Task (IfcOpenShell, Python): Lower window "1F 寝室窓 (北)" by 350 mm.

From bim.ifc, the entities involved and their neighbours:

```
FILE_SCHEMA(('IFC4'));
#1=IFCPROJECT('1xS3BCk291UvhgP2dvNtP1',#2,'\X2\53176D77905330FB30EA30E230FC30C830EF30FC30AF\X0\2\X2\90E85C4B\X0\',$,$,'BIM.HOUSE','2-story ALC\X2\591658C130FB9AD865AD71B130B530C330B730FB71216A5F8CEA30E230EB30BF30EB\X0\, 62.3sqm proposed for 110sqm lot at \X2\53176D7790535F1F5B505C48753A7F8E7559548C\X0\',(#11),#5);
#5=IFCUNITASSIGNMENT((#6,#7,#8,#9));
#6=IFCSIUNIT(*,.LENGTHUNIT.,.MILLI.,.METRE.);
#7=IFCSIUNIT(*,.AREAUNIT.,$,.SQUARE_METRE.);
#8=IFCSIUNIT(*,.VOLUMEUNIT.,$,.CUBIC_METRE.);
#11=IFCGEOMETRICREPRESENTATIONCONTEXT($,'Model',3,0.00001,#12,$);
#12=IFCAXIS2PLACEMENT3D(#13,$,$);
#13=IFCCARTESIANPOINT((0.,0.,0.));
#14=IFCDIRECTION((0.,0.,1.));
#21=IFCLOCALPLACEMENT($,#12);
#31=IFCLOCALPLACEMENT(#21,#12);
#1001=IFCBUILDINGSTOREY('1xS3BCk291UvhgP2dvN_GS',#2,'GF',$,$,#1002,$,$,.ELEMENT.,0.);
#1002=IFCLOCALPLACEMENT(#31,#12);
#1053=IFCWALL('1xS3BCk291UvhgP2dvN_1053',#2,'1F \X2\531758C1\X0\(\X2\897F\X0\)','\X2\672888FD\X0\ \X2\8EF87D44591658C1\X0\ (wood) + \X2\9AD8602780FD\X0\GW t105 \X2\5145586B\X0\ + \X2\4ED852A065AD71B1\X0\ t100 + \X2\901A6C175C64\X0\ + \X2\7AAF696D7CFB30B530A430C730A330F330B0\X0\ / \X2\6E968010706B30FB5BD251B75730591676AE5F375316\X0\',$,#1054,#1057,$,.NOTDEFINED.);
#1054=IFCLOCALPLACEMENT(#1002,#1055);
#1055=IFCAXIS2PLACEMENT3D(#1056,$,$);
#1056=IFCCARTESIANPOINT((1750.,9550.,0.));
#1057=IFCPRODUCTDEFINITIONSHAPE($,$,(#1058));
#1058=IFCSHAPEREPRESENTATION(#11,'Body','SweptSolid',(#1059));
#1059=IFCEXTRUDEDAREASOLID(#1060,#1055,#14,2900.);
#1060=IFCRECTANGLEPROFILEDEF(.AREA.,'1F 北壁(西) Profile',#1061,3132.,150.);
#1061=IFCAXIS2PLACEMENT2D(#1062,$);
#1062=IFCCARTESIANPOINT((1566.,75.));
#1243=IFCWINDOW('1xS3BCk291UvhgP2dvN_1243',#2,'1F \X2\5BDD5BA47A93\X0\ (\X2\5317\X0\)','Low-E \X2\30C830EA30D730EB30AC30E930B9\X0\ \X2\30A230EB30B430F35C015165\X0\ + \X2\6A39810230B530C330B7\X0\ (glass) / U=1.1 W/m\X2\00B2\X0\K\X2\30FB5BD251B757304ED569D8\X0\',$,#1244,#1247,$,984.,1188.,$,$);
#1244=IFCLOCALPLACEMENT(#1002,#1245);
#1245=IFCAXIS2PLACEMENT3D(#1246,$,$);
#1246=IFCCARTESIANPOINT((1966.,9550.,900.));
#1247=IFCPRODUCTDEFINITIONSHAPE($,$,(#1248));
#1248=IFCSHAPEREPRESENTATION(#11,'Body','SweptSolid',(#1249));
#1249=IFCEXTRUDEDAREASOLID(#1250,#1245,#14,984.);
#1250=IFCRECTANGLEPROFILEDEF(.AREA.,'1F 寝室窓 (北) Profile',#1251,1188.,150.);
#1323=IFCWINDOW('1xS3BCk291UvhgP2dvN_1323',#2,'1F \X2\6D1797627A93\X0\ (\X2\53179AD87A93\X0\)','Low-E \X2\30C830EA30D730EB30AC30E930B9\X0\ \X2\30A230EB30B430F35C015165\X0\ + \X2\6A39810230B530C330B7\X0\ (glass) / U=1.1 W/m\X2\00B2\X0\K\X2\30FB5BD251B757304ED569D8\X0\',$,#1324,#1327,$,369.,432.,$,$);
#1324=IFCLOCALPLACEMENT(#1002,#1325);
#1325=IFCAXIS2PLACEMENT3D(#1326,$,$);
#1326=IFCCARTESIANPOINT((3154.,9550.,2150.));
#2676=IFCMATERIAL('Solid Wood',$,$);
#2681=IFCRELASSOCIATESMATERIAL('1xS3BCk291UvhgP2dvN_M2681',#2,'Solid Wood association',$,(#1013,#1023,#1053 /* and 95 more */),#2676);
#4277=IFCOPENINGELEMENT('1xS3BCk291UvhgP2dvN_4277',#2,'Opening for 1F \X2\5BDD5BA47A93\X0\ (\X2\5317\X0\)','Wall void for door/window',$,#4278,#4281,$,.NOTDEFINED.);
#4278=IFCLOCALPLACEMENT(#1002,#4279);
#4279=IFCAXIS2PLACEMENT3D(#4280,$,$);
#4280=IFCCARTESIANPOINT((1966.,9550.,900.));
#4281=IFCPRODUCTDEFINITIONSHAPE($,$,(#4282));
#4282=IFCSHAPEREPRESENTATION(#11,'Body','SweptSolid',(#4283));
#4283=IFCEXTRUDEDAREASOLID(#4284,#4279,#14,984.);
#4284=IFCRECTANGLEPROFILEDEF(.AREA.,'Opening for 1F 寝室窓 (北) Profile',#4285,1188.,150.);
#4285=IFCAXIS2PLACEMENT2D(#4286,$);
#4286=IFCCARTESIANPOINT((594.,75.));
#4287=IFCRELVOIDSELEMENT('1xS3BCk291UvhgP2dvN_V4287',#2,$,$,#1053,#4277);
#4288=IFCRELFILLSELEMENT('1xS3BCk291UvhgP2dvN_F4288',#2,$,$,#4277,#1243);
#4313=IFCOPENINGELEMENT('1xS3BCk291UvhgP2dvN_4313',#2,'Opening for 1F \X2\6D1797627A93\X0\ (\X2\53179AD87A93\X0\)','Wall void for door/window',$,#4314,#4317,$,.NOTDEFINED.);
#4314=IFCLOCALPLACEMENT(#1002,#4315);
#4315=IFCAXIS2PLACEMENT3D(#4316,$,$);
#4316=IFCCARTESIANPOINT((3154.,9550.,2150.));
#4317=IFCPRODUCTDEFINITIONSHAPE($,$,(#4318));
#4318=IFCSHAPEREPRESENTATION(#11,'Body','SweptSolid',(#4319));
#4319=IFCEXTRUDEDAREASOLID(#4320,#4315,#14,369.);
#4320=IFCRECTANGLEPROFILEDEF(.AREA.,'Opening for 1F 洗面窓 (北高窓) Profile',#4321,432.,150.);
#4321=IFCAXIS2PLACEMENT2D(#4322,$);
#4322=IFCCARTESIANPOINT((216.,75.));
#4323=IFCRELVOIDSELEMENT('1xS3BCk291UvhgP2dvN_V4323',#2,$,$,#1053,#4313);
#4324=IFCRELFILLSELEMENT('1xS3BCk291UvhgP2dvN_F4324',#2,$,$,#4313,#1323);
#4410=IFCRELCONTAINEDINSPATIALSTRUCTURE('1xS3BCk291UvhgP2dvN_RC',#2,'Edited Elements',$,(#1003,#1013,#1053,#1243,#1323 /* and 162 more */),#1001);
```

```python
import numpy as np
import ifcopenshell
import ifcopenshell.api.geometry
import ifcopenshell.util.placement
import ifcopenshell.util.unit

model = ifcopenshell.open("bim.ifc")
unit_scale = ifcopenshell.util.unit.calculate_unit_scale(model)

window = model.by_id(1243)
opening = window.FillsVoids[0].RelatingOpeningElement
dz = -0.35 / unit_scale

shift = np.array([0.0, 0.0, dz])
# The window is not placed relative to its opening, so move both.
for product in (opening, window):
    matrix = ifcopenshell.util.placement.get_local_placement(product.ObjectPlacement)
    matrix[:3, 3] += shift
    ifcopenshell.api.geometry.edit_object_placement(model, product=product, matrix=matrix, is_si=False)

print(f"moved by {dz * unit_scale:+.3f} m")

model.write("bim_v2.ifc")
```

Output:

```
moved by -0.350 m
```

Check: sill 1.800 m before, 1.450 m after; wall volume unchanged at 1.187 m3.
